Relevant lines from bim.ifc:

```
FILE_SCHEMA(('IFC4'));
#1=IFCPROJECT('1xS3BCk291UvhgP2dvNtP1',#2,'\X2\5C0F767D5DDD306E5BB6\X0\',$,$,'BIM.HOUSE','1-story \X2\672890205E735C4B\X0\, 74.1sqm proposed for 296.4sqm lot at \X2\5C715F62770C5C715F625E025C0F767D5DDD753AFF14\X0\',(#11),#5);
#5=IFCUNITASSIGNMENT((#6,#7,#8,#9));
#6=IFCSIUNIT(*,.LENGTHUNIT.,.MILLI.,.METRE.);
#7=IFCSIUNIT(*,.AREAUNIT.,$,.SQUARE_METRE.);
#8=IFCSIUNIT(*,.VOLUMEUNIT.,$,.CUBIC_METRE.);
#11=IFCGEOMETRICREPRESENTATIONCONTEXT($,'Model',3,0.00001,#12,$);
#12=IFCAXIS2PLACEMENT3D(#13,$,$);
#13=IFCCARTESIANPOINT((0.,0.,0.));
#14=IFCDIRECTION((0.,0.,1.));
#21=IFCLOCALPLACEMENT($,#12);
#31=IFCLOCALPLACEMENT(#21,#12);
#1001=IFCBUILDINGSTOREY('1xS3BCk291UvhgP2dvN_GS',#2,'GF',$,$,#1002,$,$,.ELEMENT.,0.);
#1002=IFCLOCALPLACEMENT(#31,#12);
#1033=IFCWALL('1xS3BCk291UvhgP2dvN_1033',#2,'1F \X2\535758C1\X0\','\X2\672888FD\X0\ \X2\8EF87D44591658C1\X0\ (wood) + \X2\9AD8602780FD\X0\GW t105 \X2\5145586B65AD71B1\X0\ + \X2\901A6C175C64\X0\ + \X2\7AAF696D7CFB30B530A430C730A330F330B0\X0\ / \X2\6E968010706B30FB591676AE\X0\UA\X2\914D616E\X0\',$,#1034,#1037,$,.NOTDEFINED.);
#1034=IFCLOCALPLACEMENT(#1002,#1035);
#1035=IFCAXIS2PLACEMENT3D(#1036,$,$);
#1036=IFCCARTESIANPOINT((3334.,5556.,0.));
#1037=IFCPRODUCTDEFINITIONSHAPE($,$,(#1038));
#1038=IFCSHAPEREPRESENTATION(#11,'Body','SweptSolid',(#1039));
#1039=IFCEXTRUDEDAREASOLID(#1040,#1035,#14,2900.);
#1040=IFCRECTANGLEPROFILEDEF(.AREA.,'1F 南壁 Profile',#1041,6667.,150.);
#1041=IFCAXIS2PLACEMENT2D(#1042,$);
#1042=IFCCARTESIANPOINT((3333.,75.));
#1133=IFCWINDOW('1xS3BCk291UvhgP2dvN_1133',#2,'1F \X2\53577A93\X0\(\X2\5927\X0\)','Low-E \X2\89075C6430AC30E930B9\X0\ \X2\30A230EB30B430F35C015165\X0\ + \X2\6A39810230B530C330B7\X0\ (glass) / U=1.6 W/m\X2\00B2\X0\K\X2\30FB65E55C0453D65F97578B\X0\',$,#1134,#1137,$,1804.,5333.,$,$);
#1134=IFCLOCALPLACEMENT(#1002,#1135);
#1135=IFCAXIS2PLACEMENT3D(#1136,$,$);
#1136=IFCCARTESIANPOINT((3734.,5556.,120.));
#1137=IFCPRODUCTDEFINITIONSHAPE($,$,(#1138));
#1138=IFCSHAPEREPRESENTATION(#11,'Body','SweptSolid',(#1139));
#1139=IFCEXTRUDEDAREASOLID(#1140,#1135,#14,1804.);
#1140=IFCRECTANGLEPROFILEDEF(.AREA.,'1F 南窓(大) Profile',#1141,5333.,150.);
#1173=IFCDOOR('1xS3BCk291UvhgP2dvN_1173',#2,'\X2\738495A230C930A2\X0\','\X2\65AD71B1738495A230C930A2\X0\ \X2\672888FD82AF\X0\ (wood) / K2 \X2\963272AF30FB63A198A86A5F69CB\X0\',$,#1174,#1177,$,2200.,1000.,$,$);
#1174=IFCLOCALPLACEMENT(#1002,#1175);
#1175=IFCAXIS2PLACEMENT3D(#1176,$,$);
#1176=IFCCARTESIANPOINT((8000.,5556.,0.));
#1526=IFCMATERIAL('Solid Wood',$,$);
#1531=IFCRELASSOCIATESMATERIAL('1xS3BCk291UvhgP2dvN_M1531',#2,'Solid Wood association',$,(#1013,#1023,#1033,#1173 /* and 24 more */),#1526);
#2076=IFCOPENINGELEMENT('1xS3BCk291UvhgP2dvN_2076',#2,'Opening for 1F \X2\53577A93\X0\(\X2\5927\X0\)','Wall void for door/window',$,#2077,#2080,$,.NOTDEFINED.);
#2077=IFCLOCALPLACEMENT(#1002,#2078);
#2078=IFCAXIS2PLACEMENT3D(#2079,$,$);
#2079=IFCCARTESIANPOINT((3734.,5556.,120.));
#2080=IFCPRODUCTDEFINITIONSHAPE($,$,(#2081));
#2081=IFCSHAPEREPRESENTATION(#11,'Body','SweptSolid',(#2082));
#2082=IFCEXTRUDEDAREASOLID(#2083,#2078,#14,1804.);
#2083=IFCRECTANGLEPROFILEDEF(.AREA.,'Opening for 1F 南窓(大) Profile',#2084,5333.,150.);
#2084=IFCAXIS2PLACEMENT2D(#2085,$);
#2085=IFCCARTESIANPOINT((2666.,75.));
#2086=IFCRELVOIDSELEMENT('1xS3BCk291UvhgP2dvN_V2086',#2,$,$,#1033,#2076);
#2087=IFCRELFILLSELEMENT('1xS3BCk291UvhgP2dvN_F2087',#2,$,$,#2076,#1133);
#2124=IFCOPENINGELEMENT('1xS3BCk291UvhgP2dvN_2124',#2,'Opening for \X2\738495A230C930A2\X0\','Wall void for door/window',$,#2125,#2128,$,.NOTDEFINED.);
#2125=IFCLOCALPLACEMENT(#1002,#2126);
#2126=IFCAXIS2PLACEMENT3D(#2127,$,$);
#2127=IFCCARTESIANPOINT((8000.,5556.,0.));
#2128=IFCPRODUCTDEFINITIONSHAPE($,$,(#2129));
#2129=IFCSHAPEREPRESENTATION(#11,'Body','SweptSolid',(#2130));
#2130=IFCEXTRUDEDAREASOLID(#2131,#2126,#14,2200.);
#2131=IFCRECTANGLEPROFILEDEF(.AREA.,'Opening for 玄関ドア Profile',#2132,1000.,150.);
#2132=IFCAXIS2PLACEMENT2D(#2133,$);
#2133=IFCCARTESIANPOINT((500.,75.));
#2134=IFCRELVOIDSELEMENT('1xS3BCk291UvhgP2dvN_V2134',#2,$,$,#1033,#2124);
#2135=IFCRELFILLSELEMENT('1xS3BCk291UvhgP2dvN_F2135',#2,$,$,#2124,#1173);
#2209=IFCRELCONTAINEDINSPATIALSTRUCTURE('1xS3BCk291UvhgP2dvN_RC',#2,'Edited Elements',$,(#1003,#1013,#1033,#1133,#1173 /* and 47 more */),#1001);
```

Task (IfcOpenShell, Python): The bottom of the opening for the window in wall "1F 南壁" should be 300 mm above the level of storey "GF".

```python
import numpy as np
import ifcopenshell
import ifcopenshell.api.geometry
import ifcopenshell.geom
import ifcopenshell.util.element
import ifcopenshell.util.placement
import ifcopenshell.util.shape
import ifcopenshell.util.unit

model = ifcopenshell.open("bim.ifc")
unit_scale = ifcopenshell.util.unit.calculate_unit_scale(model)

window = model.by_guid("1xS3BCk291UvhgP2dvN_1133")
opening = window.FillsVoids[0].RelatingOpeningElement
storey = ifcopenshell.util.element.get_container(window, ifc_class="IfcBuildingStorey")
level = ifcopenshell.util.placement.get_local_placement(storey.ObjectPlacement)[2, 3]

# The opening's origin need not be at the sill, so measure its lowest point.
shape = ifcopenshell.geom.create_shape(ifcopenshell.geom.settings(), opening)
bottom = ifcopenshell.util.shape.get_shape_bottom_elevation(shape, shape.geometry) / unit_scale
dz = level + 300.0 - bottom

shift = np.array([0.0, 0.0, dz])
# The window is not placed relative to its opening, so move both.
for product in (opening, window):
    matrix = ifcopenshell.util.placement.get_local_placement(product.ObjectPlacement)
    matrix[:3, 3] += shift
    ifcopenshell.api.geometry.edit_object_placement(model, product=product, matrix=matrix, is_si=False)

print(f"moved by {dz * unit_scale:+.3f} m")

model.write("bim-out.ifc")
```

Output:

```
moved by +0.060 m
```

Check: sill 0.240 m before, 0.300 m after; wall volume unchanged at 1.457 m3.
